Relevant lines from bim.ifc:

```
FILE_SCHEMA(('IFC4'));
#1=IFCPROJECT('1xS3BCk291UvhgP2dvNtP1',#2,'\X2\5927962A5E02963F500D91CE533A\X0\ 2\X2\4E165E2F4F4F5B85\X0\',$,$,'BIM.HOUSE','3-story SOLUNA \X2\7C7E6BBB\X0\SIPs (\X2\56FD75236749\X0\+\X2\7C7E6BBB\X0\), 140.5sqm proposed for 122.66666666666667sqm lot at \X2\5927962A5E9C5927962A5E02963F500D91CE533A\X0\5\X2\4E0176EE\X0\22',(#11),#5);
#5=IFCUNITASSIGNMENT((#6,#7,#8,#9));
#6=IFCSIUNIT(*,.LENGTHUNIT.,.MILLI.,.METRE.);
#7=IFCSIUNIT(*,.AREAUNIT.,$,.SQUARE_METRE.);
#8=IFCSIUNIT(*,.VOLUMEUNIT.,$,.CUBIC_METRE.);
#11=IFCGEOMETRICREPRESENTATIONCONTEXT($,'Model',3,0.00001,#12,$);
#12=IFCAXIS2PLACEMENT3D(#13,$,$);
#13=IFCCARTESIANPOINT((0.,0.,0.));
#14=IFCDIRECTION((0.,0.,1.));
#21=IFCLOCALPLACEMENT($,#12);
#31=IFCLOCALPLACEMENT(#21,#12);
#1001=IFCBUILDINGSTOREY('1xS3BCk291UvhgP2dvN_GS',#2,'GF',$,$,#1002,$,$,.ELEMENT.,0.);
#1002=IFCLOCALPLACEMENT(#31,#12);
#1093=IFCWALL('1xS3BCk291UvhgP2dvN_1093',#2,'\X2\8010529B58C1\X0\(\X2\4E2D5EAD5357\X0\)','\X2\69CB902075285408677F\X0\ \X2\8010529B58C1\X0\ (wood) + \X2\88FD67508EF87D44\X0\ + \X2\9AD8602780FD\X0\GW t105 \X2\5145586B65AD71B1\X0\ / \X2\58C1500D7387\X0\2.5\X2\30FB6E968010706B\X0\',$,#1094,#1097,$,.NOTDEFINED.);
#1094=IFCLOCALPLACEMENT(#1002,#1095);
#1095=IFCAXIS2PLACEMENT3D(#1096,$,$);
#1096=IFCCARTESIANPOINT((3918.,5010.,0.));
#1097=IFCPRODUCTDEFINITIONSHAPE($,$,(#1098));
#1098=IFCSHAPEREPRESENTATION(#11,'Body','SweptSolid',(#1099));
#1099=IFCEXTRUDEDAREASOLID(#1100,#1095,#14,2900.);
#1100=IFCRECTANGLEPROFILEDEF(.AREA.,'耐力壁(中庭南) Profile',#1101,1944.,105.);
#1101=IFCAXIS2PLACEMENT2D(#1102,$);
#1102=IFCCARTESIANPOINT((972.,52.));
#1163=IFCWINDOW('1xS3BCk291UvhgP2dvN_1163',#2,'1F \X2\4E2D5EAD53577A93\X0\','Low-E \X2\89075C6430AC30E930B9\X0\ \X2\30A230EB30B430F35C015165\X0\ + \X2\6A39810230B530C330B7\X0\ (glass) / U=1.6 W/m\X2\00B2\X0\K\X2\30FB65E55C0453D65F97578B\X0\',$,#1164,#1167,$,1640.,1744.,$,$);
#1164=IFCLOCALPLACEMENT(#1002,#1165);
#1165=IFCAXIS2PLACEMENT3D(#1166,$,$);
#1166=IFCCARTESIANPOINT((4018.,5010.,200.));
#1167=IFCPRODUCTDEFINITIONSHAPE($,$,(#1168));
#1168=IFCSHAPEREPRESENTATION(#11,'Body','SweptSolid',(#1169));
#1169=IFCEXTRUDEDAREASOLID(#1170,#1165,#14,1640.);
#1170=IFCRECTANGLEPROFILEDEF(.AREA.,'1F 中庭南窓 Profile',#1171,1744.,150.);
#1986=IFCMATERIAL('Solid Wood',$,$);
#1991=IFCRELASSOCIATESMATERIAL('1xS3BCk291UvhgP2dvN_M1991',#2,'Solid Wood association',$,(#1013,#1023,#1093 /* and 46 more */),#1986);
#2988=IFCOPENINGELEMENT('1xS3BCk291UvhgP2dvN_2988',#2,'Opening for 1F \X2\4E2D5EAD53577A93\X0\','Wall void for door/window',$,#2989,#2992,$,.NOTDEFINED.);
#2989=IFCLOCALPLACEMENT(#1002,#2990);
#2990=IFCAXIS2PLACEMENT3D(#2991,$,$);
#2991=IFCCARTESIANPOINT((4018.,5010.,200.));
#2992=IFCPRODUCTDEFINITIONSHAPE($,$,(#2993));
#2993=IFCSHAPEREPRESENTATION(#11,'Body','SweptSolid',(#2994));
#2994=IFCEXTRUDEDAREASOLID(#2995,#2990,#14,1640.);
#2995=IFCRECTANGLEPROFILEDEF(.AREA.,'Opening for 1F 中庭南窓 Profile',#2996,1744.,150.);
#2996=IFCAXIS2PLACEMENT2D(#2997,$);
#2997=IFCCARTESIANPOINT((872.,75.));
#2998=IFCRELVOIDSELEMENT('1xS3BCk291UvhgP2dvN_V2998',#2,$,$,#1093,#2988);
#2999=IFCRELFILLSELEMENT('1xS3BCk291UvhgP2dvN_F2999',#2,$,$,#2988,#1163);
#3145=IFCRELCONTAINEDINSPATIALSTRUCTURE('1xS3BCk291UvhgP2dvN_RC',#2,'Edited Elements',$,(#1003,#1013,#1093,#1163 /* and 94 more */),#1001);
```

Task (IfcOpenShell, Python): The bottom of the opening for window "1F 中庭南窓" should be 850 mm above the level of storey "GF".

```python
import numpy as np
import ifcopenshell
import ifcopenshell.api.geometry
import ifcopenshell.geom
import ifcopenshell.util.element
import ifcopenshell.util.placement
import ifcopenshell.util.shape
import ifcopenshell.util.unit

model = ifcopenshell.open("bim.ifc")
unit_scale = ifcopenshell.util.unit.calculate_unit_scale(model)

window = model.by_id(1163)
opening = window.FillsVoids[0].RelatingOpeningElement
storey = ifcopenshell.util.element.get_container(window, ifc_class="IfcBuildingStorey")
level = ifcopenshell.util.placement.get_local_placement(storey.ObjectPlacement)[2, 3]

# The opening's origin need not be at the sill, so measure its lowest point.
shape = ifcopenshell.geom.create_shape(ifcopenshell.geom.settings(), opening)
bottom = ifcopenshell.util.shape.get_shape_bottom_elevation(shape, shape.geometry) / unit_scale
dz = level + 850.0 - bottom

shift = np.array([0.0, 0.0, dz])
# The window is not placed relative to its opening, so move both.
for product in (opening, window):
    matrix = ifcopenshell.util.placement.get_local_placement(product.ObjectPlacement)
    matrix[:3, 3] += shift
    ifcopenshell.api.geometry.edit_object_placement(model, product=product, matrix=matrix, is_si=False)

print(f"moved by {dz * unit_scale:+.3f} m")

model.write("bim_updated.ifc")
```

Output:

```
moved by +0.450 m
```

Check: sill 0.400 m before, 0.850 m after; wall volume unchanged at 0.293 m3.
